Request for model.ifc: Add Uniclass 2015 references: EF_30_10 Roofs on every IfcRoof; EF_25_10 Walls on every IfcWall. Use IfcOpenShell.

First a look at what the model holds.

```python
import ifcopenshell

model = ifcopenshell.open("model.ifc")
print(model.schema)
print("classifications:", [c.Name for c in model.by_type("IfcClassification")])
for ifc_class in ("IfcDoor", "IfcRoof", "IfcStair", "IfcWall", "IfcWindow"):
    print(ifc_class, len(model.by_type(ifc_class)))
```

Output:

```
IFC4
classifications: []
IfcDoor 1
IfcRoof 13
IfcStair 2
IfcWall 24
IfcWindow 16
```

```python
import ifcopenshell
import ifcopenshell.api.classification

model = ifcopenshell.open("model.ifc")

system = ifcopenshell.api.classification.add_classification(model, classification="Uniclass 2015")

codes = {
    "IfcRoof": ("EF_30_10", "Roofs"),
    "IfcWall": ("EF_25_10", "Walls"),
}
for ifc_class, (code, name) in codes.items():
    products = model.by_type(ifc_class)
    ifcopenshell.api.classification.add_reference(
        model, products=products, classification=system, identification=code, name=name
    )
    print(code, len(products))

model.write("model_edited.ifc")
```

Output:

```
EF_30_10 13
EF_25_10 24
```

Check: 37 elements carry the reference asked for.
